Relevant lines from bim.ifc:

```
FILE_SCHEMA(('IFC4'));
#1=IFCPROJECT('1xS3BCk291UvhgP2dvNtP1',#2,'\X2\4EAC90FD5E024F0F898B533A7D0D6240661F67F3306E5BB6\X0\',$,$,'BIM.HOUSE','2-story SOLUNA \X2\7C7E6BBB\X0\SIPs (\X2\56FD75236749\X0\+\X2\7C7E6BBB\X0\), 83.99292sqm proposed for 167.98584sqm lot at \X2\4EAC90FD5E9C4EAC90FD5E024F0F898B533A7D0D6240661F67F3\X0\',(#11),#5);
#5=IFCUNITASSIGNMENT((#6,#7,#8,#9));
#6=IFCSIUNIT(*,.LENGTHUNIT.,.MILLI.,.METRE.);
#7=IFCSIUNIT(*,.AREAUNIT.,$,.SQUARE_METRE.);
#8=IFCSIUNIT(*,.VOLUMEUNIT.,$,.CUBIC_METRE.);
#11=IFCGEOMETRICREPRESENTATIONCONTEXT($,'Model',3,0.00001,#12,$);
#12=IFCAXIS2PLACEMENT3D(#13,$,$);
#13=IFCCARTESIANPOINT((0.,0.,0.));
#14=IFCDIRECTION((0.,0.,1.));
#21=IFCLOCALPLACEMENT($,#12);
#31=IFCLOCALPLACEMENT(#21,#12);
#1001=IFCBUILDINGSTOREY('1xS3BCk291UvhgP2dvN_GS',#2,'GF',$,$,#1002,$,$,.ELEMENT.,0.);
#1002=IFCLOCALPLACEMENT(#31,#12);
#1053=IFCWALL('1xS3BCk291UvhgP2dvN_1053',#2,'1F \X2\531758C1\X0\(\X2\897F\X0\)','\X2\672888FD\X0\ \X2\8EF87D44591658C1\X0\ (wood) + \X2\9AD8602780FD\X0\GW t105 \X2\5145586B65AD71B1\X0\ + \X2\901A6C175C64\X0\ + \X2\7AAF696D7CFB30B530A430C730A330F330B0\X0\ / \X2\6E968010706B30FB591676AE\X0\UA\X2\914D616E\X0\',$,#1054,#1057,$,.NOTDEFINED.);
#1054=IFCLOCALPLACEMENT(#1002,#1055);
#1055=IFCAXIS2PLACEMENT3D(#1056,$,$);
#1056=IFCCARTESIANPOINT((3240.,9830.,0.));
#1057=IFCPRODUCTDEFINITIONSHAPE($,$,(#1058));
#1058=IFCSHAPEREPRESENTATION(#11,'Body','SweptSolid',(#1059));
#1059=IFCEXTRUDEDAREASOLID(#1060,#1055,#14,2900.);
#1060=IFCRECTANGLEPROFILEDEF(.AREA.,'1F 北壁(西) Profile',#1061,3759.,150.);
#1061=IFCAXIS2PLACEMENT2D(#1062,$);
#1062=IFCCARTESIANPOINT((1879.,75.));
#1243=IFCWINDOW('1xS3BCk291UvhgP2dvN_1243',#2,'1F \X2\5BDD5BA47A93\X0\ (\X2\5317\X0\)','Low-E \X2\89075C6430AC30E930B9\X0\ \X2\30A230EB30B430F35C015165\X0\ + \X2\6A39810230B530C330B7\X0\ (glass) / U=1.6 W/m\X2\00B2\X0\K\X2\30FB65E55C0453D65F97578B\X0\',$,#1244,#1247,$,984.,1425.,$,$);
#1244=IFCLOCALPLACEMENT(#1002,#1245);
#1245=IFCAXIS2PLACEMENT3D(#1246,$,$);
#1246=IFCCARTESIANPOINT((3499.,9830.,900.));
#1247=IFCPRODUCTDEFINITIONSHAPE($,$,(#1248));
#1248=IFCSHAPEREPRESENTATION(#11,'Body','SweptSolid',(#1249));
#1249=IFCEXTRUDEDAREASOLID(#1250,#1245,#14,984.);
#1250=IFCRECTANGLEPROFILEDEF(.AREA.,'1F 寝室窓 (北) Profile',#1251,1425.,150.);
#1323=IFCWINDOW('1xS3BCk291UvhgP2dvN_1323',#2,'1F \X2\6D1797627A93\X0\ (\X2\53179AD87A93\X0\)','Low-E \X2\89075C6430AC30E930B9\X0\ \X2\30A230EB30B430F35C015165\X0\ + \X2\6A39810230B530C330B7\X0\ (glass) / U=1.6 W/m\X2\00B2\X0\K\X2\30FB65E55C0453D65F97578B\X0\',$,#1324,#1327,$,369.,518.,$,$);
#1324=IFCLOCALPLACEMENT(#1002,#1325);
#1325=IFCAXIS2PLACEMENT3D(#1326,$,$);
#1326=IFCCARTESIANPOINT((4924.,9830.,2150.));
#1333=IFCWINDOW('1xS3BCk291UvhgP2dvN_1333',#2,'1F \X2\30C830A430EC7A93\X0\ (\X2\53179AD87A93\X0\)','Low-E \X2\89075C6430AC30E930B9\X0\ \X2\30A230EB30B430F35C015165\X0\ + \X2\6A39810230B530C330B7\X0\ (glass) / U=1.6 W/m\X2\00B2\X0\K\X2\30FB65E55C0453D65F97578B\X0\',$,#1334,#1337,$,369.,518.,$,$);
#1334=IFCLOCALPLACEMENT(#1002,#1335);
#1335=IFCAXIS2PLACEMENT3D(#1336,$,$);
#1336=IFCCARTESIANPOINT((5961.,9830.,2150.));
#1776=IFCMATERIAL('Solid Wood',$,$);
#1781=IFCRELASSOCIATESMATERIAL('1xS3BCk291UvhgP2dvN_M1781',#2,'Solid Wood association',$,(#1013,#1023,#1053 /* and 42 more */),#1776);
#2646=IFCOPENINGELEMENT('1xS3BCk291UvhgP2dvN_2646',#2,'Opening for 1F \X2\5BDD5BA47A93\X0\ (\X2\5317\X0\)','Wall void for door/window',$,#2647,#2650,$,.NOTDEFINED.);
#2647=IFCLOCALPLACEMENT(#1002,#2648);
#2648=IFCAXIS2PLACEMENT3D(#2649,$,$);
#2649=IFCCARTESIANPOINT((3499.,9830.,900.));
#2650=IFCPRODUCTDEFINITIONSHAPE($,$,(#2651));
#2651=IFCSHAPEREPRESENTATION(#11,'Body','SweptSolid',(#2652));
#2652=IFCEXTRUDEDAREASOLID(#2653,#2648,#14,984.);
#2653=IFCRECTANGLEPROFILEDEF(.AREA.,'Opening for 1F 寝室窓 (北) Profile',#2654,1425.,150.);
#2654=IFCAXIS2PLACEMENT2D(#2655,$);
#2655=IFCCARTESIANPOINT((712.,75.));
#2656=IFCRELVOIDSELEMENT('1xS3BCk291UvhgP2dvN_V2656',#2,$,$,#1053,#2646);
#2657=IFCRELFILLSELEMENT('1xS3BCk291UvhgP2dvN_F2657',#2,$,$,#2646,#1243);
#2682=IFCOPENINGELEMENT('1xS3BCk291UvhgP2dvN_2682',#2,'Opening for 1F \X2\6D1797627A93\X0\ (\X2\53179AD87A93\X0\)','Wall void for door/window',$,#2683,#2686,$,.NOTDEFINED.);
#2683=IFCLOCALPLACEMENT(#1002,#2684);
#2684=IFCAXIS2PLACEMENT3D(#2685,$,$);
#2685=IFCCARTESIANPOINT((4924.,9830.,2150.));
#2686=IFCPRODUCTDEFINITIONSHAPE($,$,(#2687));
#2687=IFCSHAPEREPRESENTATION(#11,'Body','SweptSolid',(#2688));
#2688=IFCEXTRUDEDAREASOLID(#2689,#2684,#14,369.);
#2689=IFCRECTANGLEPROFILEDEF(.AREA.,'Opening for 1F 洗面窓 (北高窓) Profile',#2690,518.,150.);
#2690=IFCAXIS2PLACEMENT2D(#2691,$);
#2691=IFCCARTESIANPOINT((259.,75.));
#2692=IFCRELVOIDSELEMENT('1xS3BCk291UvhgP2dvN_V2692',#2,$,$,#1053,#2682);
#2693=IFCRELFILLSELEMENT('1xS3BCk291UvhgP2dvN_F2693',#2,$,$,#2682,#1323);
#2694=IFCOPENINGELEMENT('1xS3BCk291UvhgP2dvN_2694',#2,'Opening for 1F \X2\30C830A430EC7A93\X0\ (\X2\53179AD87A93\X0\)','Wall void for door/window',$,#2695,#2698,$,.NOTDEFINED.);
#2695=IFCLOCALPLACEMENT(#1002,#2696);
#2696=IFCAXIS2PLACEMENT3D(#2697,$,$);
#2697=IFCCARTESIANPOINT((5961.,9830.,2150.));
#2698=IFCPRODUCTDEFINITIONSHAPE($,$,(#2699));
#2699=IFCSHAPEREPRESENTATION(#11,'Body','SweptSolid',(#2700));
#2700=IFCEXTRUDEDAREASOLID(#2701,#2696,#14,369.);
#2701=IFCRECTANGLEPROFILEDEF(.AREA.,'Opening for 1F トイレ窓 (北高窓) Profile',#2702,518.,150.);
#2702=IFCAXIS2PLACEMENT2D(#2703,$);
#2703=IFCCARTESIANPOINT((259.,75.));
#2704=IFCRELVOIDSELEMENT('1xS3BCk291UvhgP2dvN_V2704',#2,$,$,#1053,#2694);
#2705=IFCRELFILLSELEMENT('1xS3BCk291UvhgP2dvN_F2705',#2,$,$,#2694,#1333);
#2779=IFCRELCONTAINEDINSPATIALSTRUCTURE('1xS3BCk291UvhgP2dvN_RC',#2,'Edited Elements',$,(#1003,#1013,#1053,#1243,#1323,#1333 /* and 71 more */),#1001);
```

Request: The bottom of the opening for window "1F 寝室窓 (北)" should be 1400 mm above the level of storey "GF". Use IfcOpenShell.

```python
import numpy as np
import ifcopenshell
import ifcopenshell.api.geometry
import ifcopenshell.geom
import ifcopenshell.util.element
import ifcopenshell.util.placement
import ifcopenshell.util.shape
import ifcopenshell.util.unit

model = ifcopenshell.open("bim.ifc")
unit_scale = ifcopenshell.util.unit.calculate_unit_scale(model)

window = model.by_guid("1xS3BCk291UvhgP2dvN_1243")
opening = window.FillsVoids[0].RelatingOpeningElement
storey = ifcopenshell.util.element.get_container(window, ifc_class="IfcBuildingStorey")
level = ifcopenshell.util.placement.get_local_placement(storey.ObjectPlacement)[2, 3]

# The opening's origin need not be at the sill, so measure its lowest point.
shape = ifcopenshell.geom.create_shape(ifcopenshell.geom.settings(), opening)
bottom = ifcopenshell.util.shape.get_shape_bottom_elevation(shape, shape.geometry) / unit_scale
dz = level + 1.4 / unit_scale - bottom

shift = np.array([0.0, 0.0, dz])
# The window is not placed relative to its opening, so move both.
for product in (opening, window):
    matrix = ifcopenshell.util.placement.get_local_placement(product.ObjectPlacement)
    matrix[:3, 3] += shift
    ifcopenshell.api.geometry.edit_object_placement(model, product=product, matrix=matrix, is_si=False)

print(f"moved by {dz * unit_scale:+.3f} m")

model.write("bim_edited.ifc")
```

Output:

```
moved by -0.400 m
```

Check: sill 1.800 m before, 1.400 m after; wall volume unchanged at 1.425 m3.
